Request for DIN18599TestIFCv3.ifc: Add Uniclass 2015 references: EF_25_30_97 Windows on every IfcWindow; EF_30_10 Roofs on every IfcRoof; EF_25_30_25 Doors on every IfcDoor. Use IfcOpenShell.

First a look at what the model holds.

```python
import ifcopenshell

model = ifcopenshell.open("DIN18599TestIFCv3.ifc")
print(model.schema)
print("classifications:", [c.Name for c in model.by_type("IfcClassification")])
for ifc_class in ("IfcDoor", "IfcRoof", "IfcStair", "IfcWall", "IfcWindow"):
    print(ifc_class, len(model.by_type(ifc_class)))
```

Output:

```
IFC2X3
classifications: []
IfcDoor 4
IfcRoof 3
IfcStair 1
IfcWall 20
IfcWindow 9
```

```python
import ifcopenshell
import ifcopenshell.api.classification

model = ifcopenshell.open("DIN18599TestIFCv3.ifc")

# IFC2X3 requires Source and Edition and has no link from the project to the system.
system = model.create_entity("IfcClassification", Source="NBS", Edition="2015", Name="Uniclass 2015")

codes = {
    "IfcWindow": ("EF_25_30_97", "Windows"),
    "IfcRoof": ("EF_30_10", "Roofs"),
    "IfcDoor": ("EF_25_30_25", "Doors"),
}
for ifc_class, (code, name) in codes.items():
    products = model.by_type(ifc_class)
    ifcopenshell.api.classification.add_reference(
        model, products=products, classification=system, identification=code, name=name
    )
    print(code, len(products))

model.write("DIN18599TestIFCv3_edited.ifc")
```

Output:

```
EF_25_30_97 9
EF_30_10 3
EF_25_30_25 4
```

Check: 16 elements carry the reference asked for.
